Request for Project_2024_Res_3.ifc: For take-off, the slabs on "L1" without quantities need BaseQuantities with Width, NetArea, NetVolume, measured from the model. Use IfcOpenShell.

First a look at what the model holds.

```python
import ifcopenshell
import ifcopenshell.util.element
import ifcopenshell.util.unit

model = ifcopenshell.open("Project_2024_Res_3.ifc")
print(model.schema)
for unit_type in ("LENGTHUNIT", "AREAUNIT", "VOLUMEUNIT"):
    print(unit_type, ifcopenshell.util.unit.calculate_unit_scale(model, unit_type))
storey = next(s for s in model.by_type("IfcBuildingStorey") if s.Name == "L1")
slabs = [e for e in ifcopenshell.util.element.get_decomposition(storey) if e.is_a("IfcSlab")]
for e in sorted(slabs, key=lambda e: e.id()):
    print(e.id(), e.is_a(), e.Name, list(ifcopenshell.util.element.get_psets(e, qtos_only=True)), sep=" | ")
```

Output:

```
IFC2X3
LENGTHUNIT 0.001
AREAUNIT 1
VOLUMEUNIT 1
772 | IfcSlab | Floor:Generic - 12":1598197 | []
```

```python
import ifcopenshell
import ifcopenshell.api.pset
import ifcopenshell.geom
import ifcopenshell.util.element
import ifcopenshell.util.shape
import ifcopenshell.util.unit

model = ifcopenshell.open("Project_2024_Res_3.ifc")
unit_scale = ifcopenshell.util.unit.calculate_unit_scale(model)
area_scale = ifcopenshell.util.unit.calculate_unit_scale(model, "AREAUNIT")
volume_scale = ifcopenshell.util.unit.calculate_unit_scale(model, "VOLUMEUNIT")
settings = ifcopenshell.geom.settings()

storey = next(s for s in model.by_type("IfcBuildingStorey") if s.Name == "L1")
slabs = [e for e in ifcopenshell.util.element.get_decomposition(storey) if e.is_a("IfcSlab")]

for e in sorted(slabs, key=lambda e: e.id()):
    if ifcopenshell.util.element.get_psets(e, qtos_only=True, should_inherit=False):
        continue
    # Geometry comes back in metres, in the element's own axes.
    shape = ifcopenshell.geom.create_shape(settings, e)
    values = {
        "Width": ifcopenshell.util.shape.get_z(shape.geometry) / unit_scale,
        "NetArea": ifcopenshell.util.shape.get_footprint_area(shape.geometry) / area_scale,
        "NetVolume": ifcopenshell.util.shape.get_volume(shape.geometry) / volume_scale,
    }
    qto = ifcopenshell.api.pset.add_qto(model, product=e, name="BaseQuantities")
    ifcopenshell.api.pset.edit_qto(model, qto=qto, properties=values)
    print(e.id(), {k: round(v, 3) for k, v in values.items()})

model.write("Project_2024_Res_3_updated.ifc")
```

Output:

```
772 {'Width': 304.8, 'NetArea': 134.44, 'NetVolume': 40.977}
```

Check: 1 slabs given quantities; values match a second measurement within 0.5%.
